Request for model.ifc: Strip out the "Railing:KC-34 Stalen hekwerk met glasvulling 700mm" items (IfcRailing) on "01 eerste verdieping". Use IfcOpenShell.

First a look at what the model holds.

```python
import ifcopenshell
import ifcopenshell.util.element

model = ifcopenshell.open("model.ifc")
print(model.schema)
storey = next(s for s in model.by_type("IfcBuildingStorey") if s.Name == "01 eerste verdieping")
railings = [e for e in ifcopenshell.util.element.get_decomposition(storey) if e.is_a("IfcRailing")]
seen = {}
for e in railings:
    element_type = ifcopenshell.util.element.get_type(e)
    name = element_type.Name if element_type not in (None, e) else None
    seen[name] = seen.get(name, 0) + 1
for name, count in sorted(seen.items(), key=str):
    print(count, "x", name)
```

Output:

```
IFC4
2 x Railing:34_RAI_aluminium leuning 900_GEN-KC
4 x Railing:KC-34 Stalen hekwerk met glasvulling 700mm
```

```python
import ifcopenshell
import ifcopenshell.api.root
import ifcopenshell.util.element

model = ifcopenshell.open("model.ifc")

storey = next(s for s in model.by_type("IfcBuildingStorey") if s.Name == "01 eerste verdieping")
railings = [e for e in ifcopenshell.util.element.get_decomposition(storey) if e.is_a("IfcRailing")]
targets = [e for e in railings if (t := ifcopenshell.util.element.get_type(e)) not in (None, e) and t.Name == "Railing:KC-34 Stalen hekwerk met glasvulling 700mm"]

for e in targets:
    ifcopenshell.api.root.remove_product(model, product=e)
print(len(targets), "removed")

model.write("model_v2.ifc")
```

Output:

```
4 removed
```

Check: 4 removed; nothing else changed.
